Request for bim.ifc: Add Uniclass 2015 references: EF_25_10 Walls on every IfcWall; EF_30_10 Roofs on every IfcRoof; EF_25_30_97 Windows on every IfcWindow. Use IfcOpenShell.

First a look at what the model holds.

```python
import ifcopenshell

model = ifcopenshell.open("bim.ifc")
print(model.schema)
print("classifications:", [c.Name for c in model.by_type("IfcClassification")])
for ifc_class in ("IfcDoor", "IfcRoof", "IfcStair", "IfcWall", "IfcWindow"):
    print(ifc_class, len(model.by_type(ifc_class)))
```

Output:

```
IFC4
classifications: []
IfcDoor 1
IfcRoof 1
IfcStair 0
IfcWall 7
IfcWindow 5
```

```python
import ifcopenshell
import ifcopenshell.api.classification

model = ifcopenshell.open("bim.ifc")

system = ifcopenshell.api.classification.add_classification(model, classification="Uniclass 2015")

codes = {
    "IfcWall": ("EF_25_10", "Walls"),
    "IfcRoof": ("EF_30_10", "Roofs"),
    "IfcWindow": ("EF_25_30_97", "Windows"),
}
for ifc_class, (code, name) in codes.items():
    products = model.by_type(ifc_class)
    ifcopenshell.api.classification.add_reference(
        model, products=products, classification=system, identification=code, name=name
    )
    print(code, len(products))

model.write("bim_v2.ifc")
```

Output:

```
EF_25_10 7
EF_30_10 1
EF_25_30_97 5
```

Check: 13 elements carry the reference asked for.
